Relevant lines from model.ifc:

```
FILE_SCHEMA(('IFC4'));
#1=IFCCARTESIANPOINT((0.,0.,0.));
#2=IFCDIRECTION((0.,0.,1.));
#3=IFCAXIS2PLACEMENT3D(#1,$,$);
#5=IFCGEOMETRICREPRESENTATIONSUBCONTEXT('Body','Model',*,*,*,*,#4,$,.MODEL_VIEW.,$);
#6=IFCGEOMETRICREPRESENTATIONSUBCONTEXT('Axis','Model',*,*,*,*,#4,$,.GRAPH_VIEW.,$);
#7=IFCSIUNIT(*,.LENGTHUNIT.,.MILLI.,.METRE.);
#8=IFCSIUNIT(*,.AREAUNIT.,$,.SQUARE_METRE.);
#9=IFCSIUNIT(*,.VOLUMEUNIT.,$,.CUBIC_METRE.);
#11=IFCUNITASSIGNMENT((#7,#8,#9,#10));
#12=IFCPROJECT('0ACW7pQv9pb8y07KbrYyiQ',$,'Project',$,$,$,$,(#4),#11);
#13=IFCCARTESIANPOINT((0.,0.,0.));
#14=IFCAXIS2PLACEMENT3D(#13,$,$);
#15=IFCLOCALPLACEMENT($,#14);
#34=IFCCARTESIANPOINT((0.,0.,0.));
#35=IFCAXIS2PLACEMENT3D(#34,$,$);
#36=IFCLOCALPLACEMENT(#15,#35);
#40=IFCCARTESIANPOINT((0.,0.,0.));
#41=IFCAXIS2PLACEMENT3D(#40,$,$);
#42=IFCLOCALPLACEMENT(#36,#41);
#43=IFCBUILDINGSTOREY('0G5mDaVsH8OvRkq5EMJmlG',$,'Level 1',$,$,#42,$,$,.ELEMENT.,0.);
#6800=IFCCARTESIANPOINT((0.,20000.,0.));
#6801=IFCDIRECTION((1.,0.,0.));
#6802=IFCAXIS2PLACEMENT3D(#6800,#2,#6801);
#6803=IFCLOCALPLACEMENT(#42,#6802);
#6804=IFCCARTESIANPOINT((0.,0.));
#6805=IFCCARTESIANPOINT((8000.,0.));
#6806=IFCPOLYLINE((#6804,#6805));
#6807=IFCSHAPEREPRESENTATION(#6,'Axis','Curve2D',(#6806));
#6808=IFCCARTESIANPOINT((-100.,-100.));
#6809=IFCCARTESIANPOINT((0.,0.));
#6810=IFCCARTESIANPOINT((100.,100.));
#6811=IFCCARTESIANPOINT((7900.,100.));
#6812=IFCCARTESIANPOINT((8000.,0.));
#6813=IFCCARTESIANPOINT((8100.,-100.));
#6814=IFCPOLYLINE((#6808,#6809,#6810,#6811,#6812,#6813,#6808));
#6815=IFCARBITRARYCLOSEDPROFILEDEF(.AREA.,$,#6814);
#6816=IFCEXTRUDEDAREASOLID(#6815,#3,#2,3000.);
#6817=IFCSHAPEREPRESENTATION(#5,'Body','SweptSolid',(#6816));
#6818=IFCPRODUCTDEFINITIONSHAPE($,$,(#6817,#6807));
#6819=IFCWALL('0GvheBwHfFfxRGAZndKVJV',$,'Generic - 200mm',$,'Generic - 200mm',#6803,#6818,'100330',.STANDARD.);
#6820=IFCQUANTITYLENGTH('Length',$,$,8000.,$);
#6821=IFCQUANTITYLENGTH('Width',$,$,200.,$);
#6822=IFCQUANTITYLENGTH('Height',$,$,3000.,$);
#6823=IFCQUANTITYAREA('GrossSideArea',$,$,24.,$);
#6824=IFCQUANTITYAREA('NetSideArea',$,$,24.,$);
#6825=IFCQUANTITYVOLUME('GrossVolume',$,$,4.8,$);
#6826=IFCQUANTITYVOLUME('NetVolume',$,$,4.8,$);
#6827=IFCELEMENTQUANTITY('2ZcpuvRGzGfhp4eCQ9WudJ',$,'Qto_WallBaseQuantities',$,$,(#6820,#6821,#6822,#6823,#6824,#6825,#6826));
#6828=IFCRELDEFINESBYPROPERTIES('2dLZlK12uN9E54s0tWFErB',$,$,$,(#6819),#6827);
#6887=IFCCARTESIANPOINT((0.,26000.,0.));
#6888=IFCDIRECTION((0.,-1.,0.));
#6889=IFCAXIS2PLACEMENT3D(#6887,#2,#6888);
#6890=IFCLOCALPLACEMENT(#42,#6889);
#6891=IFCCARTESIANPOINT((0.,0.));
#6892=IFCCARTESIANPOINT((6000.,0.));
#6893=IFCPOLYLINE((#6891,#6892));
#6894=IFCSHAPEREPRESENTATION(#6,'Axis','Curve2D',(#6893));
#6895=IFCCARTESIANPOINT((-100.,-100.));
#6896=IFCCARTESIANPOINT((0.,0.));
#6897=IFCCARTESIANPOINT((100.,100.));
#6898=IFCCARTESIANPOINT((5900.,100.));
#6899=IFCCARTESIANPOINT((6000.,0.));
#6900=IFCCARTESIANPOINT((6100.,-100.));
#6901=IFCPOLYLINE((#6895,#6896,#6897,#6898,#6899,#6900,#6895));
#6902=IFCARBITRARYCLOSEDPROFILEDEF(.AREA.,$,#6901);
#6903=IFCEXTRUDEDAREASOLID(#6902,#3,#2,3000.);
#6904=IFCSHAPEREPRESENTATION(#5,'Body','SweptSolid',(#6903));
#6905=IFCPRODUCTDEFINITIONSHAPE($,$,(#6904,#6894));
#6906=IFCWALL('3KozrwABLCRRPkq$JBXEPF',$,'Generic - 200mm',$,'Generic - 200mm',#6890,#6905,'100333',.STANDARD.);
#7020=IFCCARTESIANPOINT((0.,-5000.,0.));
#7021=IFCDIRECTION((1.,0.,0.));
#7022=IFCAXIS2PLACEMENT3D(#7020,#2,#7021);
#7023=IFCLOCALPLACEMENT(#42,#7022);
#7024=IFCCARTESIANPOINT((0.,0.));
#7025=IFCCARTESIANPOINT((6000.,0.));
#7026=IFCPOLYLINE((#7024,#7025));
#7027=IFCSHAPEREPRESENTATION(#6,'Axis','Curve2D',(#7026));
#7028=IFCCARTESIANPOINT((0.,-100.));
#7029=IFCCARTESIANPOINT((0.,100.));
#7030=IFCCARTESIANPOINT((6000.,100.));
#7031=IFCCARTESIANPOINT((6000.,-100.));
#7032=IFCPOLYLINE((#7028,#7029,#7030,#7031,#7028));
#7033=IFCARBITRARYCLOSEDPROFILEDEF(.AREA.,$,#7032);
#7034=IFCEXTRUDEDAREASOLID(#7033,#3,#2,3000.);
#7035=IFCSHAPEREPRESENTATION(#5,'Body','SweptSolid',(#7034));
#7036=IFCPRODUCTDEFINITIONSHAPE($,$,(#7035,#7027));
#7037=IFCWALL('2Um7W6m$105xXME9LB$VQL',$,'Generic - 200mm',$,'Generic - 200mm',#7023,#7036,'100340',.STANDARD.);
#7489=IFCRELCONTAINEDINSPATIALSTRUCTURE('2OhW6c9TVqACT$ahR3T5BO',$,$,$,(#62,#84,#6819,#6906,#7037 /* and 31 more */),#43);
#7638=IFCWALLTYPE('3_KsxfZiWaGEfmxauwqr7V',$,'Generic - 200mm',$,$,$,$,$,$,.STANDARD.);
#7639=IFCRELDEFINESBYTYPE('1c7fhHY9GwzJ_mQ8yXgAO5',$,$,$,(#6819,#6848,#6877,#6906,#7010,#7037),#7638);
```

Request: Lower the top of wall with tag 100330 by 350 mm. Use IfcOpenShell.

```python
import ifcopenshell
import ifcopenshell.api.pset
import ifcopenshell.geom
import ifcopenshell.util.element
import ifcopenshell.util.representation
import ifcopenshell.util.shape
import ifcopenshell.util.unit

model = ifcopenshell.open("model.ifc")
unit_scale = ifcopenshell.util.unit.calculate_unit_scale(model)
area_scale = ifcopenshell.util.unit.calculate_unit_scale(model, "AREAUNIT")
volume_scale = ifcopenshell.util.unit.calculate_unit_scale(model, "VOLUMEUNIT")
settings = ifcopenshell.geom.settings()


def volume(element):
    """Net volume in cubic metres, openings subtracted."""
    shape = ifcopenshell.geom.create_shape(settings, element)
    return ifcopenshell.util.shape.get_volume(shape.geometry)


wall = model.by_guid("0GvheBwHfFfxRGAZndKVJV")
before = volume(wall)

body = ifcopenshell.util.representation.get_representation(wall, "Model", "Body")
solid = body.Items[0]
old_height = solid.Depth
solid.Depth -= 0.35 / unit_scale
after = volume(wall)
thickness = 0.2  # wall thickness in metres

# Update the stored height, areas and volumes.
qto = model.by_id(ifcopenshell.util.element.get_pset(wall, "Qto_WallBaseQuantities", should_inherit=False)["id"])
ifcopenshell.api.pset.edit_qto(model, qto=qto, properties={
    "Height": solid.Depth,
    "GrossSideArea": ifcopenshell.util.element.get_pset(wall, "Qto_WallBaseQuantities", "GrossSideArea") * solid.Depth / old_height,
    "NetSideArea": after / thickness / area_scale,
    "GrossVolume": ifcopenshell.util.element.get_pset(wall, "Qto_WallBaseQuantities", "GrossVolume") * solid.Depth / old_height,
    "NetVolume": after / volume_scale,
})

print(f"height {old_height:g} -> {solid.Depth:g}, volume {before:.3f} -> {after:.3f} m3")

model.write("model_rev.ifc")
```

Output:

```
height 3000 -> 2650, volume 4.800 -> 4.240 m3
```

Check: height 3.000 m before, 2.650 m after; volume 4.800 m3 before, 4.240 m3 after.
